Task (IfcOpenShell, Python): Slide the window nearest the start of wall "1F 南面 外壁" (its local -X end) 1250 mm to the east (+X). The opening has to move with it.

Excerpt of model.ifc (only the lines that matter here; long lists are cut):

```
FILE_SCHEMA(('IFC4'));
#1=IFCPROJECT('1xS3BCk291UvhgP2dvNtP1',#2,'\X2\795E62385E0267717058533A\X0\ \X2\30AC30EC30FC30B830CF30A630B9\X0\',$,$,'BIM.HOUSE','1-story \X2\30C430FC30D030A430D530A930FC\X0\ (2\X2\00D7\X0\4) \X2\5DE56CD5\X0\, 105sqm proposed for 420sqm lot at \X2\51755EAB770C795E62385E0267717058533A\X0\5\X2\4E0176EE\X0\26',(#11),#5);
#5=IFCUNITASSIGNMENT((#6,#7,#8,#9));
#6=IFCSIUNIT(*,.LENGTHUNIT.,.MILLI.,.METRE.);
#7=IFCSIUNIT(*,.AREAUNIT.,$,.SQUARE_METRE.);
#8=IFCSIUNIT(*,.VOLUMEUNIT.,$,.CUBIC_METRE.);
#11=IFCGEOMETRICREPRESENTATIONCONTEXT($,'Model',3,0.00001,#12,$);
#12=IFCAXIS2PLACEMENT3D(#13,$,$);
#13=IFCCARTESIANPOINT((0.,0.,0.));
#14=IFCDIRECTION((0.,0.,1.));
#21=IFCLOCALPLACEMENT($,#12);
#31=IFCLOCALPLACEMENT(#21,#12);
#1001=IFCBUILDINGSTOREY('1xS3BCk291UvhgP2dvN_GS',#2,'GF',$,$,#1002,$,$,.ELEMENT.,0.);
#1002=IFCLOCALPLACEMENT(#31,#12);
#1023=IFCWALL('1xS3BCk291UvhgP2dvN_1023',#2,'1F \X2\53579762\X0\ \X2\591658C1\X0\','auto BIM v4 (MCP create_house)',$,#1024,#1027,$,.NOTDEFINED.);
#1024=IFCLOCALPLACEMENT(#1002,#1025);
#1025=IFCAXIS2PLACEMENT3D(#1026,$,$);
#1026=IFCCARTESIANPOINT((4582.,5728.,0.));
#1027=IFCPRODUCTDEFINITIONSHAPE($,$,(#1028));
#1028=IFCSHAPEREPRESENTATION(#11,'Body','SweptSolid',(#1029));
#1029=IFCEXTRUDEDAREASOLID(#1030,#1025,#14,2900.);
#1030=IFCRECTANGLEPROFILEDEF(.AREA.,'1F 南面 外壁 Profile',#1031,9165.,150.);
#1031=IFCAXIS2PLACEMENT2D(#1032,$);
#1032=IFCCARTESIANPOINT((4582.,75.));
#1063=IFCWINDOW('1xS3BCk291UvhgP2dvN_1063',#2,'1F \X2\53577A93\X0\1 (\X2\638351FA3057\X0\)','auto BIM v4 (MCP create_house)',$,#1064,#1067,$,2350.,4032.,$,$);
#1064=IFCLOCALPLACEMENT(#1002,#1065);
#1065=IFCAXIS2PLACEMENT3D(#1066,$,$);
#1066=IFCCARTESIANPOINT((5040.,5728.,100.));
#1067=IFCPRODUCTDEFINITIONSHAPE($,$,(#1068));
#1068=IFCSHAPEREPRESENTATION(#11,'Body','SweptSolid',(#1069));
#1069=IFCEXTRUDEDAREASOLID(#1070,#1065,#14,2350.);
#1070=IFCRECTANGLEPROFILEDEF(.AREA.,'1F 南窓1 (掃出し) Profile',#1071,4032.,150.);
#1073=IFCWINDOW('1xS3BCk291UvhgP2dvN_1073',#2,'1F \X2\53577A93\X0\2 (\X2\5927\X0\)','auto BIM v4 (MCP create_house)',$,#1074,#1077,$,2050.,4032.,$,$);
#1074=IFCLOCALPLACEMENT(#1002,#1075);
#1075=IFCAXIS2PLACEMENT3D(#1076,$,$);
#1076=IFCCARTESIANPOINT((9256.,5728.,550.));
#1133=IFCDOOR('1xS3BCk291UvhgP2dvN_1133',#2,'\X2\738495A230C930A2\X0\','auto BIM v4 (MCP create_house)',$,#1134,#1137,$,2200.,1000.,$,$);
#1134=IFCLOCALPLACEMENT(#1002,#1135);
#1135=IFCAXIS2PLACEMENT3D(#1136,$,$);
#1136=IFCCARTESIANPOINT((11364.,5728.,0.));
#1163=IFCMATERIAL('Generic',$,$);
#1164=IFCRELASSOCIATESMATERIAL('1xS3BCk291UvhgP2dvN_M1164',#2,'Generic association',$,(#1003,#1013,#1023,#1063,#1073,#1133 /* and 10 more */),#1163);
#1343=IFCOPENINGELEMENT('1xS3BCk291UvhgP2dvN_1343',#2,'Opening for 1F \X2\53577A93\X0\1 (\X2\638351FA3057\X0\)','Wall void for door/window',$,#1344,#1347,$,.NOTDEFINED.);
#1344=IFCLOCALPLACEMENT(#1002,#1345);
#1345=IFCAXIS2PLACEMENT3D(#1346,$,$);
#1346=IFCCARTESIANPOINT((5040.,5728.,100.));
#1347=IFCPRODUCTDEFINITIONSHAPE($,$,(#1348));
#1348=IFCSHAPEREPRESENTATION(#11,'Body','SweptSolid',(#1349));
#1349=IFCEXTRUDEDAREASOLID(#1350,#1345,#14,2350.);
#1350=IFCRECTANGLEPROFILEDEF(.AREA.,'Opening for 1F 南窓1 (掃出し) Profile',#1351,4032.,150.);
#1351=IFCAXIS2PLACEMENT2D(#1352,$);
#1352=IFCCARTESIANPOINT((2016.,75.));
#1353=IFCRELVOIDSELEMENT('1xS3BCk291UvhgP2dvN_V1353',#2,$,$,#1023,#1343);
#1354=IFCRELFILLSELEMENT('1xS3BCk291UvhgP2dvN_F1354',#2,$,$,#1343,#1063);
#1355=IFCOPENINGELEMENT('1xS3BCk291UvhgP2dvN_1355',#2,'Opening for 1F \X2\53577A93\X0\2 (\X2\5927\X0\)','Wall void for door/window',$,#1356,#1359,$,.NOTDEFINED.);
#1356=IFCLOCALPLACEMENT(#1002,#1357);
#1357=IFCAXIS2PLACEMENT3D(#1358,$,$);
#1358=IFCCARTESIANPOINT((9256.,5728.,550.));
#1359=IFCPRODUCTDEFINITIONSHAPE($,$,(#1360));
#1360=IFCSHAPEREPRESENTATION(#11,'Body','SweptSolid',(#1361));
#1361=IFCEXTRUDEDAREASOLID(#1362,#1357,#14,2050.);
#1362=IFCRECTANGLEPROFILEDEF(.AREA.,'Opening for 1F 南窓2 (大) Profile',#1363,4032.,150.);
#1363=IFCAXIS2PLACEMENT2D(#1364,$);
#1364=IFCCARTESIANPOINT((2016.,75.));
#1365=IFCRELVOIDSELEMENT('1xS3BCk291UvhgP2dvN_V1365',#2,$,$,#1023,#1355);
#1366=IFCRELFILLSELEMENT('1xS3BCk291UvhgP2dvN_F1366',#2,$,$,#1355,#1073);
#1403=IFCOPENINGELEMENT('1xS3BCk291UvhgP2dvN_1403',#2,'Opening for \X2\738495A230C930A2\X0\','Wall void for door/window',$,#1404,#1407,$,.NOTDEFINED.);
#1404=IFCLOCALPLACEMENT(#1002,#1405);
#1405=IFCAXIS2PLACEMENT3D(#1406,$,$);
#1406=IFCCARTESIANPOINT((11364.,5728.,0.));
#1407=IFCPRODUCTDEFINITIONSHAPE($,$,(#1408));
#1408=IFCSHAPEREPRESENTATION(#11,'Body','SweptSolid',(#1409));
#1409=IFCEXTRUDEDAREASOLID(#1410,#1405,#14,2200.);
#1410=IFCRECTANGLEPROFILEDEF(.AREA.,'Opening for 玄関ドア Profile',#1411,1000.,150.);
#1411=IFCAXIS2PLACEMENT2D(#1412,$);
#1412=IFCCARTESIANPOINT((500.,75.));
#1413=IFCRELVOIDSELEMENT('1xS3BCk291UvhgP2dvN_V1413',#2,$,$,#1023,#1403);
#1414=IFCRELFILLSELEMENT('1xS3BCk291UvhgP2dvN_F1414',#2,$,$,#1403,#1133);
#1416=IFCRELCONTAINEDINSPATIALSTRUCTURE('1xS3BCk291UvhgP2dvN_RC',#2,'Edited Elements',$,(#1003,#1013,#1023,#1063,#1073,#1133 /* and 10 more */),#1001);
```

```python
import ifcopenshell
import ifcopenshell.api.geometry
import ifcopenshell.util.placement
import ifcopenshell.util.unit

model = ifcopenshell.open("model.ifc")
unit_scale = ifcopenshell.util.unit.calculate_unit_scale(model)

window = model.by_guid("1xS3BCk291UvhgP2dvN_1063")
opening = window.FillsVoids[0].RelatingOpeningElement
wall = opening.VoidsElements[0].RelatingBuildingElement

wall_matrix = ifcopenshell.util.placement.get_local_placement(wall.ObjectPlacement)
shift = wall_matrix[:3, 0] * 1.25 / unit_scale
before = ifcopenshell.util.placement.get_local_placement(window.ObjectPlacement)[:3, 3].copy()

# The window is not placed relative to its opening, so move both.
for product in (opening, window):
    matrix = ifcopenshell.util.placement.get_local_placement(product.ObjectPlacement)
    matrix[:3, 3] += shift
    ifcopenshell.api.geometry.edit_object_placement(model, product=product, matrix=matrix, is_si=False)

after = ifcopenshell.util.placement.get_local_placement(window.ObjectPlacement)[:3, 3]
print("window moved by", (after - before).round(3) + 0.0)

model.write("model_v2.ifc")
```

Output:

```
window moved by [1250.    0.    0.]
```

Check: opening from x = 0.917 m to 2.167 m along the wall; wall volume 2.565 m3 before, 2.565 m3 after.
